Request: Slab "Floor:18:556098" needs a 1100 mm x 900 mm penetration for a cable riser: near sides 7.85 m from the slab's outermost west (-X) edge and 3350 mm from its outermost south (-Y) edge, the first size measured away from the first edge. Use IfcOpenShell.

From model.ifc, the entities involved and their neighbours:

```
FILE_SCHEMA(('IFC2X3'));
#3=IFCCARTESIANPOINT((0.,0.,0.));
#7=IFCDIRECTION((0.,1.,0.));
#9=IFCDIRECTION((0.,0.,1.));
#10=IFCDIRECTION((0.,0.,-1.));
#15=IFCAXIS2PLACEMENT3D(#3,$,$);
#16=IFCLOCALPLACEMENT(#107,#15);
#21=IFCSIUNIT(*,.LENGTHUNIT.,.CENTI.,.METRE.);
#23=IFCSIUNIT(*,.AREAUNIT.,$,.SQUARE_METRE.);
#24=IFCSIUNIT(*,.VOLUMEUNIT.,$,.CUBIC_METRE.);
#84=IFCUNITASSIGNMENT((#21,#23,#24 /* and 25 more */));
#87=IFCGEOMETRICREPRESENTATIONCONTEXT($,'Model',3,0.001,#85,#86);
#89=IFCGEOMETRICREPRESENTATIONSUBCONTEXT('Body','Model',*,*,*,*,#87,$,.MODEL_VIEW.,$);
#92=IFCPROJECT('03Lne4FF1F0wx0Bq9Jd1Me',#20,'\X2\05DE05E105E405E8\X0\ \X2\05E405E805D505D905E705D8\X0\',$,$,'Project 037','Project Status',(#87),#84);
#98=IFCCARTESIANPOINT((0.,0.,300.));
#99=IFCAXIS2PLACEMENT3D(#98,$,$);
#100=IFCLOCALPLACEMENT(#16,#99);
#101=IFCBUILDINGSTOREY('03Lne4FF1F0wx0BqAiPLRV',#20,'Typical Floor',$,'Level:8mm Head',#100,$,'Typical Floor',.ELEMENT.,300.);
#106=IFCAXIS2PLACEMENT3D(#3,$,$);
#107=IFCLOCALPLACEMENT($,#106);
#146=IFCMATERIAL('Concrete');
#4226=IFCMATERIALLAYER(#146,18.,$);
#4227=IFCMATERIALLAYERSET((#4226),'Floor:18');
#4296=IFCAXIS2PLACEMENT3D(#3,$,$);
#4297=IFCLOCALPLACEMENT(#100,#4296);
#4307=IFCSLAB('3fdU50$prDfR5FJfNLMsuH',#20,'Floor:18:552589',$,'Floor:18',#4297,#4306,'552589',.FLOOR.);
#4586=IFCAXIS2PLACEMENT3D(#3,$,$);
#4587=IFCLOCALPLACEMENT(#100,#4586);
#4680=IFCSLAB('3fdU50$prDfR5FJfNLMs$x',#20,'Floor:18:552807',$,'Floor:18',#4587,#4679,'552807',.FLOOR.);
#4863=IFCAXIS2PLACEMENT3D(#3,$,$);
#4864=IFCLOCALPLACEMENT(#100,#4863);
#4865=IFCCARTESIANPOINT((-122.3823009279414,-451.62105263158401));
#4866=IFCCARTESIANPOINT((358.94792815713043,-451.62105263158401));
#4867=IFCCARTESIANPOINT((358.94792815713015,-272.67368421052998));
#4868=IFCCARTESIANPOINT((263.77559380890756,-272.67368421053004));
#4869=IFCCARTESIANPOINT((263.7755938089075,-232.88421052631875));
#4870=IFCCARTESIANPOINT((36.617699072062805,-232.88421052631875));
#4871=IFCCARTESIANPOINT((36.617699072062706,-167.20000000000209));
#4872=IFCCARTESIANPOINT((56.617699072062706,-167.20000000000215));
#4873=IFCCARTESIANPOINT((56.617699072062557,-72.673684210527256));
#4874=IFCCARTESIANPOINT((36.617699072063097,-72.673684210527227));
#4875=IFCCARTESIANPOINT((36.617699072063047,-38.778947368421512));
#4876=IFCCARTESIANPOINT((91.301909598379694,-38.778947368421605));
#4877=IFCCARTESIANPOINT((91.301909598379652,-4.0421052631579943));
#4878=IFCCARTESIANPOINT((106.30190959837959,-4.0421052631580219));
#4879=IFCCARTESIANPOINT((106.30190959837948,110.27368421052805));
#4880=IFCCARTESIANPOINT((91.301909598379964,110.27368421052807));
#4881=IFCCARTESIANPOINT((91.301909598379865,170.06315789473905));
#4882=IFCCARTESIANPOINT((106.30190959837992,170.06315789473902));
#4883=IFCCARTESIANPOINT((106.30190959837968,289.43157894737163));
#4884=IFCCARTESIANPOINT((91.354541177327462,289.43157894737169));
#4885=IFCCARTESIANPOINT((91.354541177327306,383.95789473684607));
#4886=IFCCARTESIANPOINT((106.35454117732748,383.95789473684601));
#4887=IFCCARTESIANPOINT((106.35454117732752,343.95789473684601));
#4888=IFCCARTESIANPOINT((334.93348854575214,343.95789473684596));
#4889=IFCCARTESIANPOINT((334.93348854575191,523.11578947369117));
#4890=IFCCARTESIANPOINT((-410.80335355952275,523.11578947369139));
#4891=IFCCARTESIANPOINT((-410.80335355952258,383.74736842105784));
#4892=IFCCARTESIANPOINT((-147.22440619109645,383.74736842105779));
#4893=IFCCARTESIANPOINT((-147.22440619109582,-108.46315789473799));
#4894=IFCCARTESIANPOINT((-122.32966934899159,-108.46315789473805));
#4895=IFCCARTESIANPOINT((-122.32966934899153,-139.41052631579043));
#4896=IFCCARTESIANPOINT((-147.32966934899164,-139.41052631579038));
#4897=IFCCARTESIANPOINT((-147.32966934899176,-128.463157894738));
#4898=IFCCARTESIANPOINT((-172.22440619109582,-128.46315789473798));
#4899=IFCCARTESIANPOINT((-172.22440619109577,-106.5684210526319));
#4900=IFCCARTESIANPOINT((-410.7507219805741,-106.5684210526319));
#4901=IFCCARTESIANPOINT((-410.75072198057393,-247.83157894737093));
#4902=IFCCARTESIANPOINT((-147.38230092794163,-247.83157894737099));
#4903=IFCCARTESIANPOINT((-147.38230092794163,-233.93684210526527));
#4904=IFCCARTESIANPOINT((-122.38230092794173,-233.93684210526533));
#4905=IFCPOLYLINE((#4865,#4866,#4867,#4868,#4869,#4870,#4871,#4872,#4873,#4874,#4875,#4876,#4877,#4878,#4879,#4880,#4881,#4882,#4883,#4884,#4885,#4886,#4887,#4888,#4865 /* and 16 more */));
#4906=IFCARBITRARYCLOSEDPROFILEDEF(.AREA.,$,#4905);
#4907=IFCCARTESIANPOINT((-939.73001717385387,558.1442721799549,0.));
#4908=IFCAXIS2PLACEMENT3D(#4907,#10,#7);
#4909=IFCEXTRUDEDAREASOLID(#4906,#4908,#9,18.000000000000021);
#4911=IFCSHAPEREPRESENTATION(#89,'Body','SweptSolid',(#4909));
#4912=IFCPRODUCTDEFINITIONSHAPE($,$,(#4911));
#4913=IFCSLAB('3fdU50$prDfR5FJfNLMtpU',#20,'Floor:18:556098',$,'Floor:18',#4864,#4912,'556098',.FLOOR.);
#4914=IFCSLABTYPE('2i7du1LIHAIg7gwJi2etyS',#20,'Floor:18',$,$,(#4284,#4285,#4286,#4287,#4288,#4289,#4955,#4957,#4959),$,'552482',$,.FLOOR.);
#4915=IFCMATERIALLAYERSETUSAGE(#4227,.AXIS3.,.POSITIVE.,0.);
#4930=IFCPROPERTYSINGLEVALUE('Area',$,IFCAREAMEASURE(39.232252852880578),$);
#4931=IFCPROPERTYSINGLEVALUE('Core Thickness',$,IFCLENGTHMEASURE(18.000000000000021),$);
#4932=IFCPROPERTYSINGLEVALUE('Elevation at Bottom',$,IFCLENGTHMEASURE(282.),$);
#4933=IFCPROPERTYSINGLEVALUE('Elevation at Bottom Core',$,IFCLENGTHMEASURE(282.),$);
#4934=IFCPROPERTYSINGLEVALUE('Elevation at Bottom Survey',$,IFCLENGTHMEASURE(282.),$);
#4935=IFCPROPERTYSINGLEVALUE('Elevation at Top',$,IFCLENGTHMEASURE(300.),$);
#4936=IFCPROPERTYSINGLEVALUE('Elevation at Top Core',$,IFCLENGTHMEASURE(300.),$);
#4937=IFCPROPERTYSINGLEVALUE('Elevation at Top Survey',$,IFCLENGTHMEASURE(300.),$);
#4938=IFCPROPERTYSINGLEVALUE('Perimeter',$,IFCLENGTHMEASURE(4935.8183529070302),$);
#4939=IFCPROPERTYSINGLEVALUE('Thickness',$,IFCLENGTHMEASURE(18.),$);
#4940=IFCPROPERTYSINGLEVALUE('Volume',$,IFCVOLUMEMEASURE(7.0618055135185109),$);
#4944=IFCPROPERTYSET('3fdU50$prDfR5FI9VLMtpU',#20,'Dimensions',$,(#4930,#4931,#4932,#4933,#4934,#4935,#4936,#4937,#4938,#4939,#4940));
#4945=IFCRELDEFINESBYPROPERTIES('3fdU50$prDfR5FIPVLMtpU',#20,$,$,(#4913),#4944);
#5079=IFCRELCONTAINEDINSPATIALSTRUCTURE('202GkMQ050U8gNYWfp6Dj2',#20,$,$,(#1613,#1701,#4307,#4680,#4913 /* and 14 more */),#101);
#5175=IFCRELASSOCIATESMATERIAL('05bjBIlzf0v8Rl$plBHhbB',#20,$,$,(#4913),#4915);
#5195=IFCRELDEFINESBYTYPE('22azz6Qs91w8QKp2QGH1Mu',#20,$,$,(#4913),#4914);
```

```python
import numpy as np
import ifcopenshell
import ifcopenshell.api.feature
import ifcopenshell.api.geometry
import ifcopenshell.api.pset
import ifcopenshell.api.root
import ifcopenshell.geom
import ifcopenshell.util.element
import ifcopenshell.util.placement
import ifcopenshell.util.representation
import ifcopenshell.util.shape
import ifcopenshell.util.unit

model = ifcopenshell.open("model.ifc")
unit_scale = ifcopenshell.util.unit.calculate_unit_scale(model)
area_scale = ifcopenshell.util.unit.calculate_unit_scale(model, "AREAUNIT")
volume_scale = ifcopenshell.util.unit.calculate_unit_scale(model, "VOLUMEUNIT")
settings = ifcopenshell.geom.settings()


def volume(element):
    """Net volume in cubic metres, openings subtracted."""
    shape = ifcopenshell.geom.create_shape(settings, element)
    return ifcopenshell.util.shape.get_volume(shape.geometry)


slab = model.by_id(4913)
before = volume(slab)

# Extent in the slab's own axes, in metres. The edges named are its -X and -Y sides.
slab_shape = ifcopenshell.geom.create_shape(settings, slab)
vertices = ifcopenshell.util.shape.get_vertices(slab_shape.geometry)
x_min, y_min, bottom = vertices.min(axis=0)
top = vertices[:, 2].max()

opening = ifcopenshell.api.root.create_entity(model, ifc_class="IfcOpeningElement", name="Cable riser opening")
context = ifcopenshell.util.representation.get_context(model, "Model", "Body", "MODEL_VIEW")
width, depth = 1.1, 0.9
outline = [(0.0, 0.0), (width, 0.0), (width, depth), (0.0, depth), (0.0, 0.0)]
# Overshoot both faces by 50 mm so the cut is clean.
shape = ifcopenshell.api.geometry.add_slab_representation(
    model, context=context, depth=top - bottom + 0.1, polyline=outline
)
ifcopenshell.api.geometry.assign_representation(model, product=opening, representation=shape)

matrix = ifcopenshell.util.placement.get_local_placement(slab.ObjectPlacement)
matrix[:, 3] = matrix @ np.append(np.array([x_min + 7.85, y_min + 3.35, bottom - 0.05]) / unit_scale, 1.0)
ifcopenshell.api.geometry.edit_object_placement(model, product=opening, matrix=matrix, is_si=False)
ifcopenshell.api.feature.add_feature(model, feature=opening, element=slab)

after = volume(slab)

# Update the slab's stored quantities.
pset = model.by_id(ifcopenshell.util.element.get_pset(slab, "Dimensions", should_inherit=False)["id"])
ifcopenshell.api.pset.edit_pset(model, pset=pset, properties={
    "Area": model.create_entity("IfcAreaMeasure", after / (top - bottom) / area_scale),
    "Volume": model.create_entity("IfcVolumeMeasure", after / volume_scale),
})

print(f"slab volume {before:.3f} -> {after:.3f} m3")

model.write("model_updated.ifc")
```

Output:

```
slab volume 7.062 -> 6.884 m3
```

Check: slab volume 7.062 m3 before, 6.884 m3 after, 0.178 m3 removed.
